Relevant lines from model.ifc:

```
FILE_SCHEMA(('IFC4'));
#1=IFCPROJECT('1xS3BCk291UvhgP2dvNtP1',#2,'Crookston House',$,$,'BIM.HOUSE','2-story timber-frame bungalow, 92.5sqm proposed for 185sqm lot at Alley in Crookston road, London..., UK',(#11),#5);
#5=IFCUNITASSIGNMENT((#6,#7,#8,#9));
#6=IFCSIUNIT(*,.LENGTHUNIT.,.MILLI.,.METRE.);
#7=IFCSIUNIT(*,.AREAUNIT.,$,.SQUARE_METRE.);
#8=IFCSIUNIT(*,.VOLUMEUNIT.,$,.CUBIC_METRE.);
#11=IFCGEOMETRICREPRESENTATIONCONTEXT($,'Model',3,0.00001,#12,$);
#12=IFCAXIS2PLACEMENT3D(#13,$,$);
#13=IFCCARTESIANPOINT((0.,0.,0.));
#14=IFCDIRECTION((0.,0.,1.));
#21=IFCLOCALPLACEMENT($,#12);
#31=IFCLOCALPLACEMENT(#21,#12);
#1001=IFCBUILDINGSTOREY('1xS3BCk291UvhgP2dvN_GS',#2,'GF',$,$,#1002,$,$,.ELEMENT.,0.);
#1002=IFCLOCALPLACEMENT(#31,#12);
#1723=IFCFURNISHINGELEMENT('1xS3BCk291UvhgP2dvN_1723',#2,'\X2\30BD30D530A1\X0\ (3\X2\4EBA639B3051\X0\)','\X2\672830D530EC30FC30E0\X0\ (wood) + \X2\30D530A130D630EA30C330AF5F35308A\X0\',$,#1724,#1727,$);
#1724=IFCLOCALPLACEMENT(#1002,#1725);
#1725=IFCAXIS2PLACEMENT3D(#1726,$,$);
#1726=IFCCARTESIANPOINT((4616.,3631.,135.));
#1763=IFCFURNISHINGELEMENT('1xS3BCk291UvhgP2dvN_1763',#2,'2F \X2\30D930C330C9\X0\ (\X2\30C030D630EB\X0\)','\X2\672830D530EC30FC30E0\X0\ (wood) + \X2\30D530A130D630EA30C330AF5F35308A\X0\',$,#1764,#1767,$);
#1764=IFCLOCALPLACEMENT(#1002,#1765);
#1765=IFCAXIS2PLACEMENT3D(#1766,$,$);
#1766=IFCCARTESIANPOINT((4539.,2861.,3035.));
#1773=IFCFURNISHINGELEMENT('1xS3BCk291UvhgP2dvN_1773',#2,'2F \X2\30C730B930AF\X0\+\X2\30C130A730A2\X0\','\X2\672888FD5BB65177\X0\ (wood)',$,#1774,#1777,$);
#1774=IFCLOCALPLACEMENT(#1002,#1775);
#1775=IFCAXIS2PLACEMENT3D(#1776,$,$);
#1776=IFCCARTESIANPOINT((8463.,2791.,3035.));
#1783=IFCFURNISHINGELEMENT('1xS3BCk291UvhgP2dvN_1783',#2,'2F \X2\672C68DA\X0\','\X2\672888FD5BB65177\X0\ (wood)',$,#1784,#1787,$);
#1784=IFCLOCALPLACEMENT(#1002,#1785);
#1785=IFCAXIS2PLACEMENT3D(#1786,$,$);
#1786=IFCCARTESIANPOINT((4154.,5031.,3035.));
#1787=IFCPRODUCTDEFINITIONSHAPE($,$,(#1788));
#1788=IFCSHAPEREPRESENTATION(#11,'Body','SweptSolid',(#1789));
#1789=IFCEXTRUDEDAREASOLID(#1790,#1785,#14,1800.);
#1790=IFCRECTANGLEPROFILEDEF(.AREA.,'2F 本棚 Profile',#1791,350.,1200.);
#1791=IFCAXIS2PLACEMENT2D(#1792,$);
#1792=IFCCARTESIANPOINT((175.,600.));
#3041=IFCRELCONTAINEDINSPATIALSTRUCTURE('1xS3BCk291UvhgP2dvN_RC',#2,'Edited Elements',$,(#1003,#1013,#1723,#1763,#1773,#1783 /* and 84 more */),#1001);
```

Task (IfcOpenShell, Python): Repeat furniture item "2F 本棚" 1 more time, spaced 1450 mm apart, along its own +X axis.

```python
import ifcopenshell
import ifcopenshell.api.geometry
import ifcopenshell.api.root
import ifcopenshell.util.element
import ifcopenshell.util.placement

model = ifcopenshell.open("model.ifc")


def reuse_history(source, copy):
    """copy_class also copies each property set's owner history, people and application; keep the originals."""
    for rel in copy.IsDefinedBy:
        if rel.is_a("IfcRelDefinesByProperties") and (history := rel.RelatingPropertyDefinition.OwnerHistory):
            rel.RelatingPropertyDefinition.OwnerHistory = source.OwnerHistory
            ifcopenshell.util.element.remove_deep2(model, history)


source = model.by_id(1783)
base = ifcopenshell.util.placement.get_local_placement(source.ObjectPlacement)
step = base[:3, 0] * 1450.0

for i in range(1, 2):
    copy = ifcopenshell.api.root.copy_class(model, product=source)
    copy.Representation = ifcopenshell.util.element.copy_deep(
        model, source.Representation, exclude=["IfcGeometricRepresentationContext", "IfcRepresentationMap"]
    )
    reuse_history(source, copy)
    matrix = base.copy()
    matrix[:3, 3] += i * step
    print("added at", matrix[:3, 3].round(3) + 0.0)
    ifcopenshell.api.geometry.edit_object_placement(model, product=copy, matrix=matrix, is_si=False)

model.write("model_updated.ifc")
```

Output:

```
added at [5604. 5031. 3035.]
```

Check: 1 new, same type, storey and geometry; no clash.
